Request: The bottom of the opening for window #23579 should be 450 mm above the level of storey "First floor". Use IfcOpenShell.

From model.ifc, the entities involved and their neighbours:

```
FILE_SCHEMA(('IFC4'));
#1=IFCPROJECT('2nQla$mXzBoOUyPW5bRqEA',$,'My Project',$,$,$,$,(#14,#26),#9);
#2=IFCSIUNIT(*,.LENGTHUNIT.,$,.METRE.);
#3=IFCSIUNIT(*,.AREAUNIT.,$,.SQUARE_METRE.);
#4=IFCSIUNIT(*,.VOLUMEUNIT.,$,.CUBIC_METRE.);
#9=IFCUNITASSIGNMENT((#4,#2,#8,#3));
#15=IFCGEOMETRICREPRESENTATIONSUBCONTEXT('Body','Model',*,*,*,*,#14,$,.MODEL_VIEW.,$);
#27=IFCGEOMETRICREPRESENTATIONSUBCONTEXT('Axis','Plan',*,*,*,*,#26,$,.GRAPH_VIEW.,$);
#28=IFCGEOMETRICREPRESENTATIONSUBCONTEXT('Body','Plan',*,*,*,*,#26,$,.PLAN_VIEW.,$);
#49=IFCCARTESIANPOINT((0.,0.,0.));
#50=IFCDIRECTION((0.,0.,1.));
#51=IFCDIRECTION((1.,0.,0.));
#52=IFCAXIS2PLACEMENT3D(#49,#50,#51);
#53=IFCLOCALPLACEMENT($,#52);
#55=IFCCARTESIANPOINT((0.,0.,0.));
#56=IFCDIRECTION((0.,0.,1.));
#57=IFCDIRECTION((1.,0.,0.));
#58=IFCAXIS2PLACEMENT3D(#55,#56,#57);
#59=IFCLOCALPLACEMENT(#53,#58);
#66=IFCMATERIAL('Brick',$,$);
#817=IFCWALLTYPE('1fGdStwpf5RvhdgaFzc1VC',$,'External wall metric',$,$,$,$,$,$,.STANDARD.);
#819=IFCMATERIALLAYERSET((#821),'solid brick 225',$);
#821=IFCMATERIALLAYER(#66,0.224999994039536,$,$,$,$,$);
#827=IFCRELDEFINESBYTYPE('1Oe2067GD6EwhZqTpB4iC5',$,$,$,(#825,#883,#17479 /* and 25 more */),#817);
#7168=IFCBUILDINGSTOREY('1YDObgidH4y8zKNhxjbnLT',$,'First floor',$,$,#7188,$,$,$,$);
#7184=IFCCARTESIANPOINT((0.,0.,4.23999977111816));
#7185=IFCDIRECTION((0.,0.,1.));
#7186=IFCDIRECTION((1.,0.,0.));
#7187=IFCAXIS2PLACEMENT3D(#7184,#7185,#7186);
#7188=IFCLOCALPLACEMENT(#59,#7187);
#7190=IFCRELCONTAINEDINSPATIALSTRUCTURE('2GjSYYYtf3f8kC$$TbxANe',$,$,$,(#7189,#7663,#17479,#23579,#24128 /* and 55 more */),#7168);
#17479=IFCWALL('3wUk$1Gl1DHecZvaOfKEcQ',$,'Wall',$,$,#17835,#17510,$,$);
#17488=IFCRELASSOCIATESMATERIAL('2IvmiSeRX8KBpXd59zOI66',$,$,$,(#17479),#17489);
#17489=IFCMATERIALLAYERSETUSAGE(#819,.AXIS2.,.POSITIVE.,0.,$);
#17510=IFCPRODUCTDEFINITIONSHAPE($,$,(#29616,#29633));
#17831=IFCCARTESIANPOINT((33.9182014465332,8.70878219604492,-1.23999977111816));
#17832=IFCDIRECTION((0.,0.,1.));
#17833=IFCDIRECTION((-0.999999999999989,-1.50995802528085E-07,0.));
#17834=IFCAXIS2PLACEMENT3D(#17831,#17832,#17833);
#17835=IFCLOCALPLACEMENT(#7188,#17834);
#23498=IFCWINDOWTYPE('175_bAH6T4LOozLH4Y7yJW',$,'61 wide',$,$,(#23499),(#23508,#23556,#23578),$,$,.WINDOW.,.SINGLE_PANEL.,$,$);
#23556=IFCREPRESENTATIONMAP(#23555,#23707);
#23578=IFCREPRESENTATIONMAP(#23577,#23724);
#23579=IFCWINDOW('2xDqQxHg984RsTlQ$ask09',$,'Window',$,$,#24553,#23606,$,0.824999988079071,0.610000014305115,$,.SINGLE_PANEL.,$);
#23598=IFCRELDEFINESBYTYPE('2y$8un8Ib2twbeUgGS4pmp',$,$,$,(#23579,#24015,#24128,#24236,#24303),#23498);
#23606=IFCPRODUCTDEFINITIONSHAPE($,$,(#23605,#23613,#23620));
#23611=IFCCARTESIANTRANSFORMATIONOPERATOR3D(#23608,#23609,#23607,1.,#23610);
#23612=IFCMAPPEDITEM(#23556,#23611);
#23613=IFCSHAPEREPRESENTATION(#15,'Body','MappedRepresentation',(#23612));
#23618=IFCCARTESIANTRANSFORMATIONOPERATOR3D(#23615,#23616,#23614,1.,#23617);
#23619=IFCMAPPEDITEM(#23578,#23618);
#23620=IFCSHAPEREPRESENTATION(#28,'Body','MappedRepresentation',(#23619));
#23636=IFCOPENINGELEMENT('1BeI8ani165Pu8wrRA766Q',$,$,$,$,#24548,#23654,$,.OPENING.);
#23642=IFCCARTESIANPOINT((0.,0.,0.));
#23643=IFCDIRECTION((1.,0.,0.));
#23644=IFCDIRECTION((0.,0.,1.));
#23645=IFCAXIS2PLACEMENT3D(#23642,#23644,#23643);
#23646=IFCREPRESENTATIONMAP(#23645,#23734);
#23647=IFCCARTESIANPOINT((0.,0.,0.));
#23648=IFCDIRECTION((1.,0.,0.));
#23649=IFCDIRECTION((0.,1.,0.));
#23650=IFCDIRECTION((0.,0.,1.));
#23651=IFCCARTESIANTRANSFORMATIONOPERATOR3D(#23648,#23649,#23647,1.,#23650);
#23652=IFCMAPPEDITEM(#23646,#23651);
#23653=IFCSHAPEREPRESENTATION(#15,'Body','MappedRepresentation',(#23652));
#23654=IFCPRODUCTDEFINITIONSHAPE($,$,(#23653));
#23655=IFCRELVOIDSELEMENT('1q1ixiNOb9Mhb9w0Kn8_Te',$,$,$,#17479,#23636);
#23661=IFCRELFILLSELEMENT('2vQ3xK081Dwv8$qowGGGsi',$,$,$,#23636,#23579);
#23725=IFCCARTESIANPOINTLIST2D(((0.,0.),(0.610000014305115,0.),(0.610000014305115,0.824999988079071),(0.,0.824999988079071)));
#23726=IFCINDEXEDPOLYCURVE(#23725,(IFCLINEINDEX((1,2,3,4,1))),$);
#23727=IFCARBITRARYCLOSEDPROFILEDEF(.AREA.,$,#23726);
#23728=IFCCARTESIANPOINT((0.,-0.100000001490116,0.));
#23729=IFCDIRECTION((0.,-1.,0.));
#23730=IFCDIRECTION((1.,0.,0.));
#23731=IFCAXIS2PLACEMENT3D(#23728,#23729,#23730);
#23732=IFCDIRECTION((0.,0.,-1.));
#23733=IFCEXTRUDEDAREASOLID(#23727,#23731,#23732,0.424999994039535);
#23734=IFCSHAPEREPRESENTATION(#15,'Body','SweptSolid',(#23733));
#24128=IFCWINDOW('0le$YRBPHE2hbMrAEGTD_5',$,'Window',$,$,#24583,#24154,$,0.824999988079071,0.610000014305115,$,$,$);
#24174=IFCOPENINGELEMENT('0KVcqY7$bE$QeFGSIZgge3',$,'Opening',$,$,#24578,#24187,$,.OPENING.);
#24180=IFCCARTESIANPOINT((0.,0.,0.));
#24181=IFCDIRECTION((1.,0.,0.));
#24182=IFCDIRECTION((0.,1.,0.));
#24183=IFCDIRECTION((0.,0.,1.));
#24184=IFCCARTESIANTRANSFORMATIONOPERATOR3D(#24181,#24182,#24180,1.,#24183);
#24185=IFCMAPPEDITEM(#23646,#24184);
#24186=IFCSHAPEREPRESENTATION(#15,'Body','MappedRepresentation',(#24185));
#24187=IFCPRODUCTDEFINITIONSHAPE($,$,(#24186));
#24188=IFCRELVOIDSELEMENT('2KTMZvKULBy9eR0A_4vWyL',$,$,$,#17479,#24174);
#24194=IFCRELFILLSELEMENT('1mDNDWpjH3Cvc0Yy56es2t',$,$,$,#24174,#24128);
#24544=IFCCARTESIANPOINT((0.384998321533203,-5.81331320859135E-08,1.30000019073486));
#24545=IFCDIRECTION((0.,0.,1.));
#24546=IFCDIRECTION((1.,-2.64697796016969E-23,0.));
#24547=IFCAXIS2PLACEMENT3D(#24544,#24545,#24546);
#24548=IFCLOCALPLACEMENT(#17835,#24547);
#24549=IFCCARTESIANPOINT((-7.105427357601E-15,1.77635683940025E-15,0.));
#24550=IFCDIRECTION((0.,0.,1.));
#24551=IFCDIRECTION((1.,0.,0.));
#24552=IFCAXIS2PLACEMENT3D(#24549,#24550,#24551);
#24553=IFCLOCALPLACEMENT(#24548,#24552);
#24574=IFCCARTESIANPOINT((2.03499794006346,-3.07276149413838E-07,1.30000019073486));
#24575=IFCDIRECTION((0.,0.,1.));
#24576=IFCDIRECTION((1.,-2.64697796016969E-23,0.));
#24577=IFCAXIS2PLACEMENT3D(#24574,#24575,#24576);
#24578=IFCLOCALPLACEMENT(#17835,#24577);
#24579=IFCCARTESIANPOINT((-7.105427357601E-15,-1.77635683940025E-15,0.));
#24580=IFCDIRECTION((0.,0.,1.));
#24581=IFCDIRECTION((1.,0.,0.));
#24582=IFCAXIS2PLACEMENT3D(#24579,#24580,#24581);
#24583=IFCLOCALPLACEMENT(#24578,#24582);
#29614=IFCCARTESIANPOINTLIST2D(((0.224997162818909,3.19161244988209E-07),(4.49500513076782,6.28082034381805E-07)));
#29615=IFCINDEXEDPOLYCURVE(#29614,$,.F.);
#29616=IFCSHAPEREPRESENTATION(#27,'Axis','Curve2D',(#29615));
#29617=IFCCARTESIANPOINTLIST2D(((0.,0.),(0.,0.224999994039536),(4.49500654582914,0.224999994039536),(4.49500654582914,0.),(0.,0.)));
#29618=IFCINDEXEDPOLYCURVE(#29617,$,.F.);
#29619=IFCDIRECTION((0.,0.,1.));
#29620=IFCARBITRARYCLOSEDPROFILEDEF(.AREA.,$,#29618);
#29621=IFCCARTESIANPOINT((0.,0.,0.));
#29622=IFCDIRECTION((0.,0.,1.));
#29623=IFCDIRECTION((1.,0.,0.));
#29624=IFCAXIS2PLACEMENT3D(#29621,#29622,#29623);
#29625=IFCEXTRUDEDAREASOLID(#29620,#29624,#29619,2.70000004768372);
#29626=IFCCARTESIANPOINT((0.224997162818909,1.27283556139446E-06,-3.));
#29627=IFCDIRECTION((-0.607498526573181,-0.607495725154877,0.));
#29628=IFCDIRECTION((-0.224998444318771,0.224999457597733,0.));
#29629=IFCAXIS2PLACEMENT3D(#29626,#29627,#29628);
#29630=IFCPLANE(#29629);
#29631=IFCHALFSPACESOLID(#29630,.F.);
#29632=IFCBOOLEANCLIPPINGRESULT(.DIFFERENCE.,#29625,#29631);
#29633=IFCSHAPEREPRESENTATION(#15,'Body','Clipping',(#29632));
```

```python
import numpy as np
import ifcopenshell
import ifcopenshell.api.geometry
import ifcopenshell.geom
import ifcopenshell.util.element
import ifcopenshell.util.placement
import ifcopenshell.util.shape
import ifcopenshell.util.unit

model = ifcopenshell.open("model.ifc")
unit_scale = ifcopenshell.util.unit.calculate_unit_scale(model)

window = model.by_guid("2xDqQxHg984RsTlQ$ask09")
opening = window.FillsVoids[0].RelatingOpeningElement
storey = ifcopenshell.util.element.get_container(window, ifc_class="IfcBuildingStorey")
level = ifcopenshell.util.placement.get_local_placement(storey.ObjectPlacement)[2, 3]

# The opening's origin need not be at the sill, so measure its lowest point.
shape = ifcopenshell.geom.create_shape(ifcopenshell.geom.settings(), opening)
bottom = ifcopenshell.util.shape.get_shape_bottom_elevation(shape, shape.geometry) / unit_scale
dz = level + 0.45 / unit_scale - bottom

shift = np.array([0.0, 0.0, dz])
# The window is placed relative to its opening, so it follows when the opening moves.
matrix = ifcopenshell.util.placement.get_local_placement(opening.ObjectPlacement)
matrix[:3, 3] += shift
ifcopenshell.api.geometry.edit_object_placement(
    model, product=opening, matrix=matrix, is_si=False, should_transform_children=True
)

print(f"moved by {dz * unit_scale:+.3f} m")

model.write("model-out.ifc")
```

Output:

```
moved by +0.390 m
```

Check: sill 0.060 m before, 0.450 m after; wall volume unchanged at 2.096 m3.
